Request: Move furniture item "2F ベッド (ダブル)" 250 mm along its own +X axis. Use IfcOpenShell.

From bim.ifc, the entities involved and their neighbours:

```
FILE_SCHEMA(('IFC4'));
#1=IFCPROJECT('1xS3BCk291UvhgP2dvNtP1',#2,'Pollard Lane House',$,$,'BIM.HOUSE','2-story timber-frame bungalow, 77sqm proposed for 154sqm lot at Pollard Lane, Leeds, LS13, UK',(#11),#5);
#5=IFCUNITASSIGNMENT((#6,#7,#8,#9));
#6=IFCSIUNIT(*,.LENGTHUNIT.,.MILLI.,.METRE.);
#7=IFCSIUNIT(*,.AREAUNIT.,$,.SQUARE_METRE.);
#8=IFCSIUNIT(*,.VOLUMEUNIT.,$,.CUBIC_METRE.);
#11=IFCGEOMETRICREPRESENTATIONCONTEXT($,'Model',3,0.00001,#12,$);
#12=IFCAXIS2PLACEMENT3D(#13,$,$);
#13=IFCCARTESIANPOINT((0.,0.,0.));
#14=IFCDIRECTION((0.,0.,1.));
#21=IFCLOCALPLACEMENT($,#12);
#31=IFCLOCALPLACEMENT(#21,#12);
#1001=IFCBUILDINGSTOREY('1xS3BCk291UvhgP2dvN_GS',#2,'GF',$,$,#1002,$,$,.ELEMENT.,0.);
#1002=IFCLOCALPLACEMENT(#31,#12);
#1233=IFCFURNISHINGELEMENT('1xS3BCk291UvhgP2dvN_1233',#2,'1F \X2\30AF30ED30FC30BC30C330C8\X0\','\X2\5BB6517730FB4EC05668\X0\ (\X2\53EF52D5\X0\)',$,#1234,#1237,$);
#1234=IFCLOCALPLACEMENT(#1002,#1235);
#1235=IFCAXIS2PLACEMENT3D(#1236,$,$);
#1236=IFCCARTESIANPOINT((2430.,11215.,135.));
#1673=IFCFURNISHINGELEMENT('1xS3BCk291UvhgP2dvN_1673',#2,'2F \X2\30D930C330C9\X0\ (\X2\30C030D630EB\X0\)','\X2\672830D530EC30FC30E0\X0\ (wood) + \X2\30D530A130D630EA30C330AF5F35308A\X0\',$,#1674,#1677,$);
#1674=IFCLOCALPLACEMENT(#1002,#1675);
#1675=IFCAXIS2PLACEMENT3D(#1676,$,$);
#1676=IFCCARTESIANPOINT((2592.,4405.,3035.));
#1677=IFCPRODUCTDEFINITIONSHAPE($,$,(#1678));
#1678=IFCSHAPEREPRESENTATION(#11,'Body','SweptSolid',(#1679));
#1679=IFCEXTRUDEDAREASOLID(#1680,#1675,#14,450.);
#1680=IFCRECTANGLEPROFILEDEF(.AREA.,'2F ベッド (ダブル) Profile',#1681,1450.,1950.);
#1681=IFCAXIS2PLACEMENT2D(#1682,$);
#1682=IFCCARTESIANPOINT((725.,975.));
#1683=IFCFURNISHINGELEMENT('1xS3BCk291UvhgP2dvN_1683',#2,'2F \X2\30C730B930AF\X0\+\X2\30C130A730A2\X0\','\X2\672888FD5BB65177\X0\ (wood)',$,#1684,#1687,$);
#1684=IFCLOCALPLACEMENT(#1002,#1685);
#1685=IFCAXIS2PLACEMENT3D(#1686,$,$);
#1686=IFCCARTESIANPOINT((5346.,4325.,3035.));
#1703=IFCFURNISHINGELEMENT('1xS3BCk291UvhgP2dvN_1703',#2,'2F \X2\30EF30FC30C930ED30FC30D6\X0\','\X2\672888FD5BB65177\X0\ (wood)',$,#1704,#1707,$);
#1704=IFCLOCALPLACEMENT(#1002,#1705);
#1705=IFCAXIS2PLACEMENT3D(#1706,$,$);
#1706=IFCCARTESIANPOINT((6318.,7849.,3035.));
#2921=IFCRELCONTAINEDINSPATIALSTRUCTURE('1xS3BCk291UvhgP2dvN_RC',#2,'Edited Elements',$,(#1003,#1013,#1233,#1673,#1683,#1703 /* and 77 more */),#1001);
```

```python
import ifcopenshell
import ifcopenshell.api.geometry
import ifcopenshell.util.placement

model = ifcopenshell.open("bim.ifc")

item = model.by_guid("1xS3BCk291UvhgP2dvN_1673")
matrix = ifcopenshell.util.placement.get_local_placement(item.ObjectPlacement)
matrix[:3, 3] += matrix[:3, 0] * 250.0
ifcopenshell.api.geometry.edit_object_placement(model, product=item, matrix=matrix, is_si=False)

print(ifcopenshell.util.placement.get_local_placement(item.ObjectPlacement).round(3) + 0.0)

model.write("bim-out.ifc")
```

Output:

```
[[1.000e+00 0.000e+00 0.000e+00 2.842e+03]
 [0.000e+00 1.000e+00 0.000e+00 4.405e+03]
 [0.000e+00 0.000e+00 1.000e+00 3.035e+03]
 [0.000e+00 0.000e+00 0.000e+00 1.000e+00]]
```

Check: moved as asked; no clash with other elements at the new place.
